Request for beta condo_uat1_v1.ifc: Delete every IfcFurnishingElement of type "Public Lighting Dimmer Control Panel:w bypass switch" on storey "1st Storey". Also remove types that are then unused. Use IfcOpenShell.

First a look at what the model holds.

```python
import ifcopenshell
import ifcopenshell.util.element

model = ifcopenshell.open("beta condo_uat1_v1.ifc")
print(model.schema)
storey = next(s for s in model.by_type("IfcBuildingStorey") if s.Name == "1st Storey")
furniture = [e for e in ifcopenshell.util.element.get_decomposition(storey) if e.is_a("IfcFurnishingElement")]
seen = {}
for e in furniture:
    element_type = ifcopenshell.util.element.get_type(e)
    name = element_type.Name if element_type not in (None, e) else None
    seen[name] = seen.get(name, 0) + 1
for name, count in sorted(seen.items(), key=str):
    print(count, "x", name)
```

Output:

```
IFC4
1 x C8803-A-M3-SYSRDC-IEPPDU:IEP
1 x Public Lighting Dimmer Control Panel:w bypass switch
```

```python
import ifcopenshell
import ifcopenshell.api.root
import ifcopenshell.util.element

model = ifcopenshell.open("beta condo_uat1_v1.ifc")

storey = next(s for s in model.by_type("IfcBuildingStorey") if s.Name == "1st Storey")
furniture = [e for e in ifcopenshell.util.element.get_decomposition(storey) if e.is_a("IfcFurnishingElement")]
targets = [e for e in furniture if (t := ifcopenshell.util.element.get_type(e)) not in (None, e) and t.Name == "Public Lighting Dimmer Control Panel:w bypass switch"]
types = {ifcopenshell.util.element.get_type(e) for e in targets} - {None, *targets}

for e in targets:
    ifcopenshell.api.root.remove_product(model, product=e)
print(len(targets), "removed")

unused = [t for t in types if not ifcopenshell.util.element.get_types(t)]
for t in unused:
    ifcopenshell.api.root.remove_product(model, product=t)
print(len(unused), "unused types removed")

model.write("beta condo_uat1_v1-out.ifc")
```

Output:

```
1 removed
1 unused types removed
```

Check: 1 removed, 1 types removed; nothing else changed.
